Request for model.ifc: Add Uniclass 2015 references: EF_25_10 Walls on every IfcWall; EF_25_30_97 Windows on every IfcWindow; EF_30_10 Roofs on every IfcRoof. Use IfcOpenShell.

First a look at what the model holds.

```python
import ifcopenshell

model = ifcopenshell.open("model.ifc")
print(model.schema)
print("classifications:", [c.Name for c in model.by_type("IfcClassification")])
for ifc_class in ("IfcDoor", "IfcRoof", "IfcStair", "IfcWall", "IfcWindow"):
    print(ifc_class, len(model.by_type(ifc_class)))
```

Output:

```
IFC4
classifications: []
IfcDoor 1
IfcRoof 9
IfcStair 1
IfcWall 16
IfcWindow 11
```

```python
import ifcopenshell
import ifcopenshell.api.classification

model = ifcopenshell.open("model.ifc")

system = ifcopenshell.api.classification.add_classification(model, classification="Uniclass 2015")

codes = {
    "IfcWall": ("EF_25_10", "Walls"),
    "IfcWindow": ("EF_25_30_97", "Windows"),
    "IfcRoof": ("EF_30_10", "Roofs"),
}
for ifc_class, (code, name) in codes.items():
    products = model.by_type(ifc_class)
    ifcopenshell.api.classification.add_reference(
        model, products=products, classification=system, identification=code, name=name
    )
    print(code, len(products))

model.write("model_updated.ifc")
```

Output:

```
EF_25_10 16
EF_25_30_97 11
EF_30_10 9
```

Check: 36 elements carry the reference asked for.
